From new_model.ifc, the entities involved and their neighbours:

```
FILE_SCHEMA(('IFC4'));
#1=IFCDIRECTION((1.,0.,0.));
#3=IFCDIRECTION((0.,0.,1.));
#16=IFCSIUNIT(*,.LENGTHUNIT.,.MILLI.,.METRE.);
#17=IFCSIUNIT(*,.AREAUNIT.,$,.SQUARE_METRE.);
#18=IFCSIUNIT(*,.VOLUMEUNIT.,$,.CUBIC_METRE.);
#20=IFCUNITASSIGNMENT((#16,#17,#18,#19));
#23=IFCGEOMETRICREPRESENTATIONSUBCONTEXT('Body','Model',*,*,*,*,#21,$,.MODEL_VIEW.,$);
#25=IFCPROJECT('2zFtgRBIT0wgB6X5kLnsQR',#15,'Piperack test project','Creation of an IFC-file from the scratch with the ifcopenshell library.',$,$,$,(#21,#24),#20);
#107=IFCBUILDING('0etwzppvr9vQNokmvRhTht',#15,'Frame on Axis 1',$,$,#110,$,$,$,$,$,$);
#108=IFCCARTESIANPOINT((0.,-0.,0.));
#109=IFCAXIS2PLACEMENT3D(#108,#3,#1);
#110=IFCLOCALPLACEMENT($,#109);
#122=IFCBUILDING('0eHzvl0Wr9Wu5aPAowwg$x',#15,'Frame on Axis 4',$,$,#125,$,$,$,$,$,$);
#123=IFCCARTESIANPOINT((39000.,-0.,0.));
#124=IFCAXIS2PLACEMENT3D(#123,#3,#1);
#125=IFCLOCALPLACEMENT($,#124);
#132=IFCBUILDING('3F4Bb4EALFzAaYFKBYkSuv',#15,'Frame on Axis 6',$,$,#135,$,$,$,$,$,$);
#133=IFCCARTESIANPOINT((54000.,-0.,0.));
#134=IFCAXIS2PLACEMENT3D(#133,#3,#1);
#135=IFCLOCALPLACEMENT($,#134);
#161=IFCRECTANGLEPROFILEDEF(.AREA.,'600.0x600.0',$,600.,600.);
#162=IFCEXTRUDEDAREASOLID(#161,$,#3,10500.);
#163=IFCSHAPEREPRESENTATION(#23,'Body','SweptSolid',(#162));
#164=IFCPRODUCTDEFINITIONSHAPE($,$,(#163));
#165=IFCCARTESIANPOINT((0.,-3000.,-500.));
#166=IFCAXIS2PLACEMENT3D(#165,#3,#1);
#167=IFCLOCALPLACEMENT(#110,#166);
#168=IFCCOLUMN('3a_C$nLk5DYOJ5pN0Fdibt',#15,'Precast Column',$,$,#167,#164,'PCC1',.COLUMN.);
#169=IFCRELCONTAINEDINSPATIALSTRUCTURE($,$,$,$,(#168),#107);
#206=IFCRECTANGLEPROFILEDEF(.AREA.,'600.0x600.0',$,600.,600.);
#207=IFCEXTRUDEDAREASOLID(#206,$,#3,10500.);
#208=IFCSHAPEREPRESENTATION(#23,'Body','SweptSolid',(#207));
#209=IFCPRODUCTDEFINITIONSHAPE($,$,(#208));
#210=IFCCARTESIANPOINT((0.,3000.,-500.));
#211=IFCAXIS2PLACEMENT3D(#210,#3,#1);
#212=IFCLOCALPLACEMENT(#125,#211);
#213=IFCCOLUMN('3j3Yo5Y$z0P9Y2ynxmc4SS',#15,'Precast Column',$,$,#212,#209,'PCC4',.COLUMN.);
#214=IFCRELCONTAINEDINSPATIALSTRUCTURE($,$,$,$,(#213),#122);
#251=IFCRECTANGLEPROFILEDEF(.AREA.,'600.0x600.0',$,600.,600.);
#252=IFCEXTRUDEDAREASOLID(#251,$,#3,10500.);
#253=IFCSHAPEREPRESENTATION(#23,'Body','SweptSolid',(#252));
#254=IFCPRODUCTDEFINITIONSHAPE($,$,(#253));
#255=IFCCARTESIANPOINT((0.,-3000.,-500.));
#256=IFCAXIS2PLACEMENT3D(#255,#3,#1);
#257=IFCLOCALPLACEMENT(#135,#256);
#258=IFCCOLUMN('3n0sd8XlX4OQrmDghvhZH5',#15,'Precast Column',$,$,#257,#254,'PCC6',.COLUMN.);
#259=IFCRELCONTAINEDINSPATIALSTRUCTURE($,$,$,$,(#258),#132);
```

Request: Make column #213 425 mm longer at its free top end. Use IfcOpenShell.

```python
import ifcopenshell
import ifcopenshell.util.representation
import ifcopenshell.util.unit

model = ifcopenshell.open("new_model.ifc")
unit_scale = ifcopenshell.util.unit.calculate_unit_scale(model)

member = model.by_guid("3j3Yo5Y$z0P9Y2ynxmc4SS")
change = 0.425 / unit_scale

# The extrusion runs towards the end named, so only its depth changes.
body = ifcopenshell.util.representation.get_representation(member, "Model", "Body")
solid = body.Items[0]
old_length = solid.Depth
solid.Depth += change

print(f"length {old_length:g} -> {solid.Depth:g}")

model.write("new_model_updated.ifc")
```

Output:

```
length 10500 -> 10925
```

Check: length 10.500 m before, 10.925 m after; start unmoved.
